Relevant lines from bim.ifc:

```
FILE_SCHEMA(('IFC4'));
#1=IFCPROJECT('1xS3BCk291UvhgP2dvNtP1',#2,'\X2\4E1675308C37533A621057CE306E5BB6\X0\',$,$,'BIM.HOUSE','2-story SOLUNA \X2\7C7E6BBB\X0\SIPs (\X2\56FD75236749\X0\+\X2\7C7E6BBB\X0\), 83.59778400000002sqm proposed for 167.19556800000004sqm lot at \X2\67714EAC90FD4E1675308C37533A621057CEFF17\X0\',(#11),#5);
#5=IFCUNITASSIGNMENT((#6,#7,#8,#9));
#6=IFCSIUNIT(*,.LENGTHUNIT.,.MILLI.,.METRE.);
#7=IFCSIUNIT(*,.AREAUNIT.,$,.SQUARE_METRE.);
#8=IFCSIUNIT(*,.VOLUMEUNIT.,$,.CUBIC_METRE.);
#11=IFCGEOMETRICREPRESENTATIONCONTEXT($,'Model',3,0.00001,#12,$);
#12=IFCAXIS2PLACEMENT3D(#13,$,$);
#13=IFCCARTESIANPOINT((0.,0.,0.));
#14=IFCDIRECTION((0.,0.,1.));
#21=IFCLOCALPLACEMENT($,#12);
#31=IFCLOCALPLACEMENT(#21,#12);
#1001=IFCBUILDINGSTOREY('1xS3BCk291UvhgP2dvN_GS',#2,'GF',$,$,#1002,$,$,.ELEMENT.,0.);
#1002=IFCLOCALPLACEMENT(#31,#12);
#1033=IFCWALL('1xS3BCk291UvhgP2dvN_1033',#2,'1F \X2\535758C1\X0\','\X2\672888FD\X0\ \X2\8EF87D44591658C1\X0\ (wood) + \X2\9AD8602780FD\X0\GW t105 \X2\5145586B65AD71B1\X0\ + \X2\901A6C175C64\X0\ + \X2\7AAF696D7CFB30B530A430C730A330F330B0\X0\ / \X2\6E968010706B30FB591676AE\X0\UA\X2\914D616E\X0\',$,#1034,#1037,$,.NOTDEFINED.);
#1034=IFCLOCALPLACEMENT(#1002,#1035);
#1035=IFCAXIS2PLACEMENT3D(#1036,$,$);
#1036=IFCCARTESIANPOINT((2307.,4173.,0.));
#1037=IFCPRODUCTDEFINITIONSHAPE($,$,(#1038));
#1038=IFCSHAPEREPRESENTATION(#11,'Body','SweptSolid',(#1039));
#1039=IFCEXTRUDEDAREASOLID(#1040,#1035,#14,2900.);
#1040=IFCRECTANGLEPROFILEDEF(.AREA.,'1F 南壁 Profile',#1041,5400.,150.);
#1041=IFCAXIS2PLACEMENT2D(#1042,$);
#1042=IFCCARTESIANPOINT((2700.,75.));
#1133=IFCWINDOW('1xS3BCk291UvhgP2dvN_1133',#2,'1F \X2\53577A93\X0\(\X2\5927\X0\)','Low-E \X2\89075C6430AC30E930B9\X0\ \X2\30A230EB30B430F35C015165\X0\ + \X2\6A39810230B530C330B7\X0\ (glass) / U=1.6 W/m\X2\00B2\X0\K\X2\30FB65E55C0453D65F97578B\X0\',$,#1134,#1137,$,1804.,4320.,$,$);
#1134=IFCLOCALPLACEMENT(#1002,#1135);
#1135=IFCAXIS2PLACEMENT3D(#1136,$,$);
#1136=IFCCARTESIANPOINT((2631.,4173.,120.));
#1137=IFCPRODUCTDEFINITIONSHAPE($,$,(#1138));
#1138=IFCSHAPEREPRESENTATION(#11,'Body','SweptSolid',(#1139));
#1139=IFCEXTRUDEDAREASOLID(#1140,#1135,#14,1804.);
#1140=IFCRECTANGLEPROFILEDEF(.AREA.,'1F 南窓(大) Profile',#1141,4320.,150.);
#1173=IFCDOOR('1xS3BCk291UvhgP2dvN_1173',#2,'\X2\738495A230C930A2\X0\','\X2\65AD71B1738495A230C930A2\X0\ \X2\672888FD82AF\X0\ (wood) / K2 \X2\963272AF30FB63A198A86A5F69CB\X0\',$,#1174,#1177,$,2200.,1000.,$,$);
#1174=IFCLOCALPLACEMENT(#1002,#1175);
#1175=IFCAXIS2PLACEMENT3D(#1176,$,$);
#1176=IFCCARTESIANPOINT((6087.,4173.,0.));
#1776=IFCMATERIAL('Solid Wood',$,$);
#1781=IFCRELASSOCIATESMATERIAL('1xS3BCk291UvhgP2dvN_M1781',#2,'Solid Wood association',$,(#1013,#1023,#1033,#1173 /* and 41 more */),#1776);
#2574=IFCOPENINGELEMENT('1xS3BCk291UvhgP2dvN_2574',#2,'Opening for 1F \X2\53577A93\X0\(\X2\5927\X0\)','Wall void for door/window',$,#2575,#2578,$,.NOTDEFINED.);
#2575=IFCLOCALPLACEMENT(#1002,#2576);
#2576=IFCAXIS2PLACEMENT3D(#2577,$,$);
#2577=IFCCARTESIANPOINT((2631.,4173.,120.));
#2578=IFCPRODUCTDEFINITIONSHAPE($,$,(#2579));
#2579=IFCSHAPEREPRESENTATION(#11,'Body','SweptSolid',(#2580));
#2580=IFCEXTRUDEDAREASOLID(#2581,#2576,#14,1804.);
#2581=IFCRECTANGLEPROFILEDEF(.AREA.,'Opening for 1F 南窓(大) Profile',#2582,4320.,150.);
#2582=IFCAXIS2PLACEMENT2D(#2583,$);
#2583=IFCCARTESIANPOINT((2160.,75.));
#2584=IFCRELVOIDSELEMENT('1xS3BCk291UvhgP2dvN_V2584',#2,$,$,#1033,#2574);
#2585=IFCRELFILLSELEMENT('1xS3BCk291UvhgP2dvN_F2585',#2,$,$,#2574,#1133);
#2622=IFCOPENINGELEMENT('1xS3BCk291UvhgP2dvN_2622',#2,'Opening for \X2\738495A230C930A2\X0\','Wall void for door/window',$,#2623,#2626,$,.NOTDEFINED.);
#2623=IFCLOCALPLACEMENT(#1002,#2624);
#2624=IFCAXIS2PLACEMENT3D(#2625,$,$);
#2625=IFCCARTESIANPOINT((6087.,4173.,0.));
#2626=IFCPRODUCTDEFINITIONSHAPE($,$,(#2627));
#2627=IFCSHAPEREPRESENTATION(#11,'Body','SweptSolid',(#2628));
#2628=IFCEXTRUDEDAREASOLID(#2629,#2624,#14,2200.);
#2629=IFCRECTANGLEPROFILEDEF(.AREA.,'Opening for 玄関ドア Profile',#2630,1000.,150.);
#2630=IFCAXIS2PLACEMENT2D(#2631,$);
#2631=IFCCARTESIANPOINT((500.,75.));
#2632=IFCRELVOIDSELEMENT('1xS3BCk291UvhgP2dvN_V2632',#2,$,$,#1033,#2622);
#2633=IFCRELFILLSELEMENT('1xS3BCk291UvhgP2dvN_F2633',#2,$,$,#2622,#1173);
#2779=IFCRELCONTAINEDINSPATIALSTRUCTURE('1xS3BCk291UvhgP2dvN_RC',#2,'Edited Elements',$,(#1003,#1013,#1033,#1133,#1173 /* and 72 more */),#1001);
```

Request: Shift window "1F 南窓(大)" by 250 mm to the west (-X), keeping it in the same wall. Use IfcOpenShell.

```python
import ifcopenshell
import ifcopenshell.api.geometry
import ifcopenshell.util.placement

model = ifcopenshell.open("bim.ifc")

window = model.by_guid("1xS3BCk291UvhgP2dvN_1133")
opening = window.FillsVoids[0].RelatingOpeningElement
wall = opening.VoidsElements[0].RelatingBuildingElement

wall_matrix = ifcopenshell.util.placement.get_local_placement(wall.ObjectPlacement)
shift = wall_matrix[:3, 0] * -250.0
before = ifcopenshell.util.placement.get_local_placement(window.ObjectPlacement)[:3, 3].copy()

# The window is not placed relative to its opening, so move both.
for product in (opening, window):
    matrix = ifcopenshell.util.placement.get_local_placement(product.ObjectPlacement)
    matrix[:3, 3] += shift
    ifcopenshell.api.geometry.edit_object_placement(model, product=product, matrix=matrix, is_si=False)

after = ifcopenshell.util.placement.get_local_placement(window.ObjectPlacement)[:3, 3]
print("window moved by", (after - before).round(3) + 0.0)

model.write("bim_rev.ifc")
```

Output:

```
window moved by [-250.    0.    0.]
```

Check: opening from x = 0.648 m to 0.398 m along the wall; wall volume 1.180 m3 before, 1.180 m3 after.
